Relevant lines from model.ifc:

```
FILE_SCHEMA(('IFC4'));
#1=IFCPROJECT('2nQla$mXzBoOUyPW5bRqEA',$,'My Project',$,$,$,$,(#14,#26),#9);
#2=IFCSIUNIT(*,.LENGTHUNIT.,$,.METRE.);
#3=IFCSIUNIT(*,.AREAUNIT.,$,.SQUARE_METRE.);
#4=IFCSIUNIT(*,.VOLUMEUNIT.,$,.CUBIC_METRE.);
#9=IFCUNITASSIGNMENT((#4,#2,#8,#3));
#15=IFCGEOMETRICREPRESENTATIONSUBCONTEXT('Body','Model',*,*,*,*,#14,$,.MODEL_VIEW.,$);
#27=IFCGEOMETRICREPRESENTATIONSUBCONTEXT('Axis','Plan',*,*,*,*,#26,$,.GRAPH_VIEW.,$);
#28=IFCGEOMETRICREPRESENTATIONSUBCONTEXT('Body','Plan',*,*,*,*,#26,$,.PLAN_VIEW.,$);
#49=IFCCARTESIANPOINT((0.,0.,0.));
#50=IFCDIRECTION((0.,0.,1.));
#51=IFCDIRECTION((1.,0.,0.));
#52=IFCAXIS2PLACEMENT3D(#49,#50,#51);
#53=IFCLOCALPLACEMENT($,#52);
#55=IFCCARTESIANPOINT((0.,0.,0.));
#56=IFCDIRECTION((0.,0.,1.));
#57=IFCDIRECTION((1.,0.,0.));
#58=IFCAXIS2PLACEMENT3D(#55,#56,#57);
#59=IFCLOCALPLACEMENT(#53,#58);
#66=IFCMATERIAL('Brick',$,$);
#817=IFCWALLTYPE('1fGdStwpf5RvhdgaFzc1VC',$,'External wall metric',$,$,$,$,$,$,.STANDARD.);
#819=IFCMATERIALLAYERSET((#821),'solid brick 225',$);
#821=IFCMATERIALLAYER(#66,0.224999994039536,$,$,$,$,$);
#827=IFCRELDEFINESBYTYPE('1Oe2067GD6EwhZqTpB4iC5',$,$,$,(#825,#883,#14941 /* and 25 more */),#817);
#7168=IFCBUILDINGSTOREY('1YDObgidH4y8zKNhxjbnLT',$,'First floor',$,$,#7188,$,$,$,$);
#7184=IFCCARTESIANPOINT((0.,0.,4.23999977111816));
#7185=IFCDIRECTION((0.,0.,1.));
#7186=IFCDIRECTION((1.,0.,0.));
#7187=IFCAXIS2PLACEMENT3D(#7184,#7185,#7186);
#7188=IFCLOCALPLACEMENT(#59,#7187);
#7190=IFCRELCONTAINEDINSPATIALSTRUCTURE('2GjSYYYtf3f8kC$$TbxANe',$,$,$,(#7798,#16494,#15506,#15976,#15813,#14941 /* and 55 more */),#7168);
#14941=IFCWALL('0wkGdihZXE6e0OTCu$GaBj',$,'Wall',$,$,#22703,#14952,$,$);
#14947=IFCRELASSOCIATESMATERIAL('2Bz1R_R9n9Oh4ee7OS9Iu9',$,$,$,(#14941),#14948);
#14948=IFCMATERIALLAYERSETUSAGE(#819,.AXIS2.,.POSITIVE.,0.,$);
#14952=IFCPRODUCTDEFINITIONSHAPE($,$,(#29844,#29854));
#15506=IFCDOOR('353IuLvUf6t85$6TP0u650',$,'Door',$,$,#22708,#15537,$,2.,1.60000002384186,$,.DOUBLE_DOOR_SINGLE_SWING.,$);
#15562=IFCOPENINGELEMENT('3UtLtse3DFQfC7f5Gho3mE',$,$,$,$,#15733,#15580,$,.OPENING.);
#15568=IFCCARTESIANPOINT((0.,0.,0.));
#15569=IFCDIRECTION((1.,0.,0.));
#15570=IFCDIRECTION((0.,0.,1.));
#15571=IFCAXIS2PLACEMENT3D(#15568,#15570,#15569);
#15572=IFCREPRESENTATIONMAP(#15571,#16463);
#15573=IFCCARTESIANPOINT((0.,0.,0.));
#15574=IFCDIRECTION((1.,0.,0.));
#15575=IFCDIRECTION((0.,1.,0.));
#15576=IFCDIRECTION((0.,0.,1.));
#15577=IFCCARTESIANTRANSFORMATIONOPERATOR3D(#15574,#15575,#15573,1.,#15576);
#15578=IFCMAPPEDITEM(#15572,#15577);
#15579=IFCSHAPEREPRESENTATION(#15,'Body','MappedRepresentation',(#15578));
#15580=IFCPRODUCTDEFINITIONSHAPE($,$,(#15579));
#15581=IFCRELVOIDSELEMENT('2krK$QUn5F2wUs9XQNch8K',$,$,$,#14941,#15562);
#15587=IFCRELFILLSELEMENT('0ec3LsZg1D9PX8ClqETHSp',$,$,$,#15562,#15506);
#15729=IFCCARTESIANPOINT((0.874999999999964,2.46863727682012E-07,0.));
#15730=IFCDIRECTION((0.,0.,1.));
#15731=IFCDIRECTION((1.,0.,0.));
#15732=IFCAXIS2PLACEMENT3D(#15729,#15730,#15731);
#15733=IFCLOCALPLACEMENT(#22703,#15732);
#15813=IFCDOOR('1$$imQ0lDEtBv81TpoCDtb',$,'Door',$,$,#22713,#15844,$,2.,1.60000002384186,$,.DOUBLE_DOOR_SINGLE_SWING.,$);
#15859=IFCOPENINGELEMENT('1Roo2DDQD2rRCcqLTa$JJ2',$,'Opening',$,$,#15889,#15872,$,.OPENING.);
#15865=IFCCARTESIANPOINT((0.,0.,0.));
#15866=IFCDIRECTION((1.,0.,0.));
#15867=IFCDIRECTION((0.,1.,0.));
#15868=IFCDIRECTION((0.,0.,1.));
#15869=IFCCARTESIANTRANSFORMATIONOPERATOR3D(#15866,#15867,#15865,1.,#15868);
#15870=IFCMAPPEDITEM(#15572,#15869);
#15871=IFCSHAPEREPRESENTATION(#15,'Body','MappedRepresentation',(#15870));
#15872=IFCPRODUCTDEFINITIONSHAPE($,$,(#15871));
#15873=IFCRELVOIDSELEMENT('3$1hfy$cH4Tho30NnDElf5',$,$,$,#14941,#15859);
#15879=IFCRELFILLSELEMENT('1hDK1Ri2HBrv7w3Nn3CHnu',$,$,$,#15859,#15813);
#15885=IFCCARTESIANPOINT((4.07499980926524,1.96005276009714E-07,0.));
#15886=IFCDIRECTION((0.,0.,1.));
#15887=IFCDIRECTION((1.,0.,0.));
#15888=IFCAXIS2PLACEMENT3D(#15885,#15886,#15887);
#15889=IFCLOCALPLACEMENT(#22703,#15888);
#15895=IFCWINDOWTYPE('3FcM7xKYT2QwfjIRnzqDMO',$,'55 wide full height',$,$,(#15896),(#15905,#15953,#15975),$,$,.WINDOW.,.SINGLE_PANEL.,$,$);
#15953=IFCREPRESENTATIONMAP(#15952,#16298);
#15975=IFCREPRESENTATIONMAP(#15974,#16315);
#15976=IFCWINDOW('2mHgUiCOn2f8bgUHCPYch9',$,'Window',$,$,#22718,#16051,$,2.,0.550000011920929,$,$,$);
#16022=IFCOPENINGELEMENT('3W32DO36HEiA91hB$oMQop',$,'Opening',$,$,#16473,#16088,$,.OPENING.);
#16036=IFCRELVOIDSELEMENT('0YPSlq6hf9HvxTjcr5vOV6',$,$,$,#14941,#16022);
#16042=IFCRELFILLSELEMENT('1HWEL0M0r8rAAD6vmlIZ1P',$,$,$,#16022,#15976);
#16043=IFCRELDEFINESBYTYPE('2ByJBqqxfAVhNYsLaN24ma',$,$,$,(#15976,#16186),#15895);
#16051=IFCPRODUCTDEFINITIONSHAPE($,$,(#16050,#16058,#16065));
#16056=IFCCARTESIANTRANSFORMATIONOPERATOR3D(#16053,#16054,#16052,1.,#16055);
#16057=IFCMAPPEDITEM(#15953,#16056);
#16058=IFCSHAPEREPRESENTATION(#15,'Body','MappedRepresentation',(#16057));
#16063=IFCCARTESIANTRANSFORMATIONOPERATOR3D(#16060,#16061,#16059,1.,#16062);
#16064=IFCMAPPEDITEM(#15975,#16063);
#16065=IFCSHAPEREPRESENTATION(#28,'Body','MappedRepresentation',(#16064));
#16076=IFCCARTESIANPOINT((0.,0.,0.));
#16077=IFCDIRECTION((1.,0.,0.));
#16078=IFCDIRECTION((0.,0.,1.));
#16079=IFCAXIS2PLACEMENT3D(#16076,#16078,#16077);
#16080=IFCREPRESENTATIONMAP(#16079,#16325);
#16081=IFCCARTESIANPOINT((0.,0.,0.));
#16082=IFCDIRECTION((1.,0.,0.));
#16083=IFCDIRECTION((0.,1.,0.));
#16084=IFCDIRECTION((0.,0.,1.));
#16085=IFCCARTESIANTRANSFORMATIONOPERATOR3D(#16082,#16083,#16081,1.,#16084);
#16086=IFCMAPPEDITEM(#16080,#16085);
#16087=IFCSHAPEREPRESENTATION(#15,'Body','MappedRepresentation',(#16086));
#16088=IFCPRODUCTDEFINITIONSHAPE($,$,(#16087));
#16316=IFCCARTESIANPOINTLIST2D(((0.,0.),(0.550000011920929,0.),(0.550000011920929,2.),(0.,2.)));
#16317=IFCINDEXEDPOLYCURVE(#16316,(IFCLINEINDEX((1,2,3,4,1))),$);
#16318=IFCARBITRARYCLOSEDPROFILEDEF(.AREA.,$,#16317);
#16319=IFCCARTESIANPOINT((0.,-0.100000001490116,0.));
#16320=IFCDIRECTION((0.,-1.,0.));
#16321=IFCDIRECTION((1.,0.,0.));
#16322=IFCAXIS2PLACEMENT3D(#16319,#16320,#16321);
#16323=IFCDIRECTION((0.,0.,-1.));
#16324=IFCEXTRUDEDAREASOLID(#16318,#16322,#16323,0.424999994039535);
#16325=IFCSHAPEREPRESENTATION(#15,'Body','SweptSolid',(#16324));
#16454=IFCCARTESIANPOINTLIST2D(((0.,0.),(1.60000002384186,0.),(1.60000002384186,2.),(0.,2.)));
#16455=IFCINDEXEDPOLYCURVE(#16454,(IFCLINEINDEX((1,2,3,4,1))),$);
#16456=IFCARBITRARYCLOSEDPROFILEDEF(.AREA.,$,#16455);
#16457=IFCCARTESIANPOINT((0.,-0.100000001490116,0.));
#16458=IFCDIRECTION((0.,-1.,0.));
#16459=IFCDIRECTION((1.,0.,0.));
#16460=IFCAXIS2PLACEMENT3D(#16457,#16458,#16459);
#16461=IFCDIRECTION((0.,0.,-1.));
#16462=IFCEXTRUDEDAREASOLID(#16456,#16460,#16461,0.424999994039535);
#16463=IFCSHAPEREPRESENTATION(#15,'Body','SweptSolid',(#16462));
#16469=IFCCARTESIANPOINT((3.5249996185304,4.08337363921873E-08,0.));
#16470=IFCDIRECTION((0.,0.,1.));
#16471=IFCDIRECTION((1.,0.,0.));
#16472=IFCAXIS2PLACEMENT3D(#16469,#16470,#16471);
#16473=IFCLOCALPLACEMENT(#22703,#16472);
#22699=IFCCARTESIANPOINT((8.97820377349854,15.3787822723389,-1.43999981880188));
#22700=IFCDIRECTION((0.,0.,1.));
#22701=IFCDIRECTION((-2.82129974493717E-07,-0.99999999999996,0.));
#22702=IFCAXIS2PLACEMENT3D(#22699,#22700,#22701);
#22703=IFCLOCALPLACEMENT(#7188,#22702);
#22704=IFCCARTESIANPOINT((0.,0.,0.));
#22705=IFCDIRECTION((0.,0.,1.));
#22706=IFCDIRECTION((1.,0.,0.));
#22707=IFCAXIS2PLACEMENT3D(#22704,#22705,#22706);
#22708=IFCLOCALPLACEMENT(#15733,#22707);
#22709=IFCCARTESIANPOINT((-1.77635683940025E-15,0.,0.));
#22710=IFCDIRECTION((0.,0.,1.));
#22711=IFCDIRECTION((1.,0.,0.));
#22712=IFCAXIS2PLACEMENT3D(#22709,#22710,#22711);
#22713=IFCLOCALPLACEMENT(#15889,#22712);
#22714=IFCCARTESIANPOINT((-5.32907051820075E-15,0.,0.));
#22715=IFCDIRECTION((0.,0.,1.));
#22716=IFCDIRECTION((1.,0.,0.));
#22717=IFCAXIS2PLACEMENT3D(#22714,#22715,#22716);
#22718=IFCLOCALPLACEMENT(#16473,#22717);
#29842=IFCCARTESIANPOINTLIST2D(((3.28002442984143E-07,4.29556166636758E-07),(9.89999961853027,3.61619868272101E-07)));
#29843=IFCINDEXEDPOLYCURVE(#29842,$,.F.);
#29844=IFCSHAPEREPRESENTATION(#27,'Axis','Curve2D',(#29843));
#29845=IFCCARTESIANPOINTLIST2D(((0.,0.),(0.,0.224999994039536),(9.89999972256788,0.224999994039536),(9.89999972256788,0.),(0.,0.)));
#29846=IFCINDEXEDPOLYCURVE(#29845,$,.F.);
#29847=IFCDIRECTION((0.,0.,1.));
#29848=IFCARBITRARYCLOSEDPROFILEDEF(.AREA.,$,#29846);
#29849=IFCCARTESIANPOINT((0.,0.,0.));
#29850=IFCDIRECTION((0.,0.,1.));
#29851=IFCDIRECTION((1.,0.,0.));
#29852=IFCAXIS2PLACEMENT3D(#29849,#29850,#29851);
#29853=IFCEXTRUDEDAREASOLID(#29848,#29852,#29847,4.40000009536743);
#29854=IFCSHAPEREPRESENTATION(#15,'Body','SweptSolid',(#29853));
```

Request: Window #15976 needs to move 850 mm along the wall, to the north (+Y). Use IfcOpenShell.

```python
import ifcopenshell
import ifcopenshell.api.geometry
import ifcopenshell.util.placement
import ifcopenshell.util.unit

model = ifcopenshell.open("model.ifc")
unit_scale = ifcopenshell.util.unit.calculate_unit_scale(model)

window = model.by_id(15976)
opening = window.FillsVoids[0].RelatingOpeningElement
wall = opening.VoidsElements[0].RelatingBuildingElement

wall_matrix = ifcopenshell.util.placement.get_local_placement(wall.ObjectPlacement)
shift = wall_matrix[:3, 0] * -0.85 / unit_scale
before = ifcopenshell.util.placement.get_local_placement(window.ObjectPlacement)[:3, 3].copy()

# The window is placed relative to its opening, so it follows when the opening moves.
matrix = ifcopenshell.util.placement.get_local_placement(opening.ObjectPlacement)
matrix[:3, 3] += shift
ifcopenshell.api.geometry.edit_object_placement(
    model, product=opening, matrix=matrix, is_si=False, should_transform_children=True
)

after = ifcopenshell.util.placement.get_local_placement(window.ObjectPlacement)[:3, 3]
print("window moved by", (after - before).round(3) + 0.0)

model.write("model_rev.ifc")
```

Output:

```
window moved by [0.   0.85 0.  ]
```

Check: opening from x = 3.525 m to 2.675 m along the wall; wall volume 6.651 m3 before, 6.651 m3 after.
